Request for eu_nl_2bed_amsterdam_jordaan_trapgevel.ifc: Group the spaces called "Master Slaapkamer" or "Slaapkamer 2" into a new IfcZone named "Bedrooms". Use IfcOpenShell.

First a look at what the model holds.

```python
import ifcopenshell

model = ifcopenshell.open("eu_nl_2bed_amsterdam_jordaan_trapgevel.ifc")
print(model.schema)
seen = {}
for space in model.by_type("IfcSpace"):
    seen[space.LongName] = seen.get(space.LongName, 0) + 1
for name, count in sorted(seen.items(), key=str):
    print(count, "x", name)
print("zones:", [z.Name for z in model.by_type("IfcZone")][:20])
```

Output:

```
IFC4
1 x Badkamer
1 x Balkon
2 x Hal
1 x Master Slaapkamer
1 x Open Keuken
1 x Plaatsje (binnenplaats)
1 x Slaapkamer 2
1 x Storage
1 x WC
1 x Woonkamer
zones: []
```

```python
import ifcopenshell
import ifcopenshell.api.group
import ifcopenshell.api.root

model = ifcopenshell.open("eu_nl_2bed_amsterdam_jordaan_trapgevel.ifc")

names = {"Master Slaapkamer", "Slaapkamer 2"}
spaces = [s for s in model.by_type("IfcSpace") if s.LongName in names]

zone = ifcopenshell.api.root.create_entity(model, ifc_class="IfcZone", name="Bedrooms")
ifcopenshell.api.group.assign_group(model, products=spaces, group=zone)
print(len(spaces), "spaces in", zone.Name)

model.write("eu_nl_2bed_amsterdam_jordaan_trapgevel_v2.ifc")
```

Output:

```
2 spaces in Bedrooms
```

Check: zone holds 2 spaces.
